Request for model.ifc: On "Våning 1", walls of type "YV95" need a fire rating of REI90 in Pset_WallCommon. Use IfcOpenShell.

First a look at what the model holds.

```python
import ifcopenshell
import ifcopenshell.util.element

model = ifcopenshell.open("model.ifc")
print(model.schema)
storey = next(s for s in model.by_type("IfcBuildingStorey") if s.Name == "Våning 1")
walls = [e for e in ifcopenshell.util.element.get_decomposition(storey) if e.is_a("IfcWall")]
seen = {}
for e in walls:
    element_type = ifcopenshell.util.element.get_type(e)
    key = (element_type.Name if element_type != e and element_type else None, ifcopenshell.util.element.get_pset(e, "Pset_WallCommon", "FireRating"))
    seen[key] = seen.get(key, 0) + 1
for (name, value), count in sorted(seen.items(), key=str):
    print(count, "x", name, "|", value)
```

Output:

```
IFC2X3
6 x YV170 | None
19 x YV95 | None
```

```python
import ifcopenshell
import ifcopenshell.api.pset
import ifcopenshell.util.element

model = ifcopenshell.open("model.ifc")

storey = next(s for s in model.by_type("IfcBuildingStorey") if s.Name == "Våning 1")
walls = [e for e in ifcopenshell.util.element.get_decomposition(storey) if e.is_a("IfcWall")]

count = 0
for e in walls:
    element_type = ifcopenshell.util.element.get_type(e)
    if element_type in (None, e) or element_type.Name != "YV95":
        continue
    # add_pset returns the element's existing set when there is one.
    pset = ifcopenshell.api.pset.add_pset(model, product=e, name="Pset_WallCommon")
    ifcopenshell.api.pset.edit_pset(model, pset=pset, properties={"FireRating": "REI90"})
    count += 1

print(count, "walls updated")

model.write("model_v2.ifc")
```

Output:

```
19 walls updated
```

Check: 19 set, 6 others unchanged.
